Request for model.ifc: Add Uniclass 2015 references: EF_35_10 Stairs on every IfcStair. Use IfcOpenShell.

First a look at what the model holds.

```python
import ifcopenshell

model = ifcopenshell.open("model.ifc")
print(model.schema)
print("classifications:", [c.Name for c in model.by_type("IfcClassification")])
for ifc_class in ("IfcDoor", "IfcRoof", "IfcStair", "IfcWall", "IfcWindow"):
    print(ifc_class, len(model.by_type(ifc_class)))
```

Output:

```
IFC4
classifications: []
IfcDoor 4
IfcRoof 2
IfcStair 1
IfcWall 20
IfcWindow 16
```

```python
import ifcopenshell
import ifcopenshell.api.classification

model = ifcopenshell.open("model.ifc")

system = ifcopenshell.api.classification.add_classification(model, classification="Uniclass 2015")

codes = {
    "IfcStair": ("EF_35_10", "Stairs"),
}
for ifc_class, (code, name) in codes.items():
    products = model.by_type(ifc_class)
    ifcopenshell.api.classification.add_reference(
        model, products=products, classification=system, identification=code, name=name
    )
    print(code, len(products))

model.write("model-out.ifc")
```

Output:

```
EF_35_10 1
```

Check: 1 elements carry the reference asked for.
